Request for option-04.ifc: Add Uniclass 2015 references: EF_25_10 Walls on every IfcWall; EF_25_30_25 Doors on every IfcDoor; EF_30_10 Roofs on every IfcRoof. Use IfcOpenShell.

First a look at what the model holds.

```python
import ifcopenshell

model = ifcopenshell.open("option-04.ifc")
print(model.schema)
print("classifications:", [c.Name for c in model.by_type("IfcClassification")])
for ifc_class in ("IfcDoor", "IfcRoof", "IfcStair", "IfcWall", "IfcWindow"):
    print(ifc_class, len(model.by_type(ifc_class)))
```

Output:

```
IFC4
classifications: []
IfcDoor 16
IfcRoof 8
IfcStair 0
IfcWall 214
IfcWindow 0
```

```python
import ifcopenshell
import ifcopenshell.api.classification

model = ifcopenshell.open("option-04.ifc")

system = ifcopenshell.api.classification.add_classification(model, classification="Uniclass 2015")

codes = {
    "IfcWall": ("EF_25_10", "Walls"),
    "IfcDoor": ("EF_25_30_25", "Doors"),
    "IfcRoof": ("EF_30_10", "Roofs"),
}
for ifc_class, (code, name) in codes.items():
    products = model.by_type(ifc_class)
    ifcopenshell.api.classification.add_reference(
        model, products=products, classification=system, identification=code, name=name
    )
    print(code, len(products))

model.write("option-04_v2.ifc")
```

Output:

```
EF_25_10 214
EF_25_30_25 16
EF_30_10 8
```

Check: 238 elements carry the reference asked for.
